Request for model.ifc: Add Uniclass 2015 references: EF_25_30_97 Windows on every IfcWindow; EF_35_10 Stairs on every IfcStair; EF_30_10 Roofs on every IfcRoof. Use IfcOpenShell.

First a look at what the model holds.

```python
import ifcopenshell

model = ifcopenshell.open("model.ifc")
print(model.schema)
print("classifications:", [c.Name for c in model.by_type("IfcClassification")])
for ifc_class in ("IfcDoor", "IfcRoof", "IfcStair", "IfcWall", "IfcWindow"):
    print(ifc_class, len(model.by_type(ifc_class)))
```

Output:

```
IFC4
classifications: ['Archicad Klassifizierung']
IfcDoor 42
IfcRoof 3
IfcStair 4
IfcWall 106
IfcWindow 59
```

```python
import ifcopenshell
import ifcopenshell.api.classification

model = ifcopenshell.open("model.ifc")

system = ifcopenshell.api.classification.add_classification(model, classification="Uniclass 2015")

codes = {
    "IfcWindow": ("EF_25_30_97", "Windows"),
    "IfcStair": ("EF_35_10", "Stairs"),
    "IfcRoof": ("EF_30_10", "Roofs"),
}
for ifc_class, (code, name) in codes.items():
    products = model.by_type(ifc_class)
    ifcopenshell.api.classification.add_reference(
        model, products=products, classification=system, identification=code, name=name
    )
    print(code, len(products))

model.write("model_rev.ifc")
```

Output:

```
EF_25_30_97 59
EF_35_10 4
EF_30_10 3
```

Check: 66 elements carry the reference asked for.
